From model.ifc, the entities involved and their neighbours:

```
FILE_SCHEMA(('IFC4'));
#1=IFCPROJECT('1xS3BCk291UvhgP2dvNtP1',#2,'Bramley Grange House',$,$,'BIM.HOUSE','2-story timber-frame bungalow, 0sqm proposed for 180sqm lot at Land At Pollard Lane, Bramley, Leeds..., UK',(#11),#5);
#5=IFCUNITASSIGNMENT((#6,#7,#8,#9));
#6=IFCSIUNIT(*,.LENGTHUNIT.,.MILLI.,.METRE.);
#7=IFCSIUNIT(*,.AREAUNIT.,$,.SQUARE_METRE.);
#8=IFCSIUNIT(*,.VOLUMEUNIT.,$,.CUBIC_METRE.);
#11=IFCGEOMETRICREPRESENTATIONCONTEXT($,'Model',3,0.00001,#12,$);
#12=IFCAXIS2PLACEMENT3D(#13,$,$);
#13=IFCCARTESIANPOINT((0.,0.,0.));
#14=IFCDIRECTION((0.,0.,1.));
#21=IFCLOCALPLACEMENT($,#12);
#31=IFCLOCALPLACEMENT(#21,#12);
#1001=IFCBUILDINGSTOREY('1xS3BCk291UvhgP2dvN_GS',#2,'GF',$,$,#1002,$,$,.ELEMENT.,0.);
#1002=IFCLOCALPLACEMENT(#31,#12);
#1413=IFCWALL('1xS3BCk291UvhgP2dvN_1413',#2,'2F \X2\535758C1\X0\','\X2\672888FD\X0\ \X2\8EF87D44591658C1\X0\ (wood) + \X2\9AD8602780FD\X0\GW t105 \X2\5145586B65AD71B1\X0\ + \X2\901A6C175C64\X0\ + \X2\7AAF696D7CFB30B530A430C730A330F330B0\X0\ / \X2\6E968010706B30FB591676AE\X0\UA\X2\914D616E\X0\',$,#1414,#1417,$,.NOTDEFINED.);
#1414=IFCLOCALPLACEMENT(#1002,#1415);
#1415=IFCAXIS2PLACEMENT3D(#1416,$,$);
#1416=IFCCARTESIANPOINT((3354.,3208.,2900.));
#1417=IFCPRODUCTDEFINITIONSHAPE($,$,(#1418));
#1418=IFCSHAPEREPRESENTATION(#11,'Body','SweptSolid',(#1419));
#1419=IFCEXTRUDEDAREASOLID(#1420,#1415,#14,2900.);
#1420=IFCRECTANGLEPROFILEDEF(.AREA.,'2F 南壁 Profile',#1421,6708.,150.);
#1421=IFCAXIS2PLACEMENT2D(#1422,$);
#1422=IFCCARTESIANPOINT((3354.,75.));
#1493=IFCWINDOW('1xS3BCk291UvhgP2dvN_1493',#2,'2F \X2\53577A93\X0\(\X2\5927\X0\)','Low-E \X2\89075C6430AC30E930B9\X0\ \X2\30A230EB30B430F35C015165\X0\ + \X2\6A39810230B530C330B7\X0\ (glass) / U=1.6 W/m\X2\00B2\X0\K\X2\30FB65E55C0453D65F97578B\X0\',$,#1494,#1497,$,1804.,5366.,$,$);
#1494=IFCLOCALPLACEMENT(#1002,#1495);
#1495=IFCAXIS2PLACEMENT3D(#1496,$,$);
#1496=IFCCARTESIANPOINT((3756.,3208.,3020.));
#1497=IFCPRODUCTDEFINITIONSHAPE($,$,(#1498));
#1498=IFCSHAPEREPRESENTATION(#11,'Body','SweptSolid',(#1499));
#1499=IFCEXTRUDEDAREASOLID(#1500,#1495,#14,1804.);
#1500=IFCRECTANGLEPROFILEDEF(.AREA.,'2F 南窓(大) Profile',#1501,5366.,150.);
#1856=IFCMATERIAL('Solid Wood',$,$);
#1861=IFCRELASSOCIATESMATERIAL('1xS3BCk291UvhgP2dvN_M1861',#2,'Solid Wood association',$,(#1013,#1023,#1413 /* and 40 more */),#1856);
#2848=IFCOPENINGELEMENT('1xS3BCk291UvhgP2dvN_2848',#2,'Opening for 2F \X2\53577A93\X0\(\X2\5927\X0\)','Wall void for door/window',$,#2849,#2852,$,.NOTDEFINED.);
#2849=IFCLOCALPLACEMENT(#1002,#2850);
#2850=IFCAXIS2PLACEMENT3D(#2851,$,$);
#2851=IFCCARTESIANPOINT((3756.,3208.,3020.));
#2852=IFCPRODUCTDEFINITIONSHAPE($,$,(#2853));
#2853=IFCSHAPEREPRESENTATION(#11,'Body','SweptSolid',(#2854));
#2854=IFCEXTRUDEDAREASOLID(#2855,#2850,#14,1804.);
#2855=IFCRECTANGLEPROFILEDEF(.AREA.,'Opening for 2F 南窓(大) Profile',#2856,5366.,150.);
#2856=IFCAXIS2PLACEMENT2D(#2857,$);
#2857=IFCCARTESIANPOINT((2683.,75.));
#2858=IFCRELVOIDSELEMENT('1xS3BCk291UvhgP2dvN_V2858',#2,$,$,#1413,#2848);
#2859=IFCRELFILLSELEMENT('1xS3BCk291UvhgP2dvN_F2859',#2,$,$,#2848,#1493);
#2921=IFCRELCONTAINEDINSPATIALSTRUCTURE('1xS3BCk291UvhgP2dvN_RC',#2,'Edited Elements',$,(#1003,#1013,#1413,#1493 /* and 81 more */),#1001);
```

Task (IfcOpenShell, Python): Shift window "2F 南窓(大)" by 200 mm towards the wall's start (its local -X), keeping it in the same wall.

```python
import ifcopenshell
import ifcopenshell.api.geometry
import ifcopenshell.util.placement
import ifcopenshell.util.unit

model = ifcopenshell.open("model.ifc")
unit_scale = ifcopenshell.util.unit.calculate_unit_scale(model)

window = model.by_id(1493)
opening = window.FillsVoids[0].RelatingOpeningElement
wall = opening.VoidsElements[0].RelatingBuildingElement

wall_matrix = ifcopenshell.util.placement.get_local_placement(wall.ObjectPlacement)
shift = wall_matrix[:3, 0] * -0.2 / unit_scale
before = ifcopenshell.util.placement.get_local_placement(window.ObjectPlacement)[:3, 3].copy()

# The window is not placed relative to its opening, so move both.
for product in (opening, window):
    matrix = ifcopenshell.util.placement.get_local_placement(product.ObjectPlacement)
    matrix[:3, 3] += shift
    ifcopenshell.api.geometry.edit_object_placement(model, product=product, matrix=matrix, is_si=False)

after = ifcopenshell.util.placement.get_local_placement(window.ObjectPlacement)[:3, 3]
print("window moved by", (after - before).round(3) + 0.0)

model.write("model_v2.ifc")
```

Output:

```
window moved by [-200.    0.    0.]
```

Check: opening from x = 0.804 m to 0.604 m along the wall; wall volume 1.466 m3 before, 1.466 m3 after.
